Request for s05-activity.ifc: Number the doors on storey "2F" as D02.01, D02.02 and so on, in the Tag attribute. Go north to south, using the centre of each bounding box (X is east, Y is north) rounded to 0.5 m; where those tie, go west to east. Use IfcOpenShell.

First a look at what the model holds.

```python
import ifcopenshell
import ifcopenshell.util.element
import ifcopenshell.util.placement

model = ifcopenshell.open("s05-activity.ifc")
print(model.schema)
storey = next(s for s in model.by_type("IfcBuildingStorey") if s.Name == "2F")
doors = [e for e in ifcopenshell.util.element.get_decomposition(storey) if e.is_a("IfcDoor")]
for e in sorted(doors, key=lambda e: e.id()):
    origin = ifcopenshell.util.placement.get_local_placement(e.ObjectPlacement)[:3, 3]
    print(e.id(), e.Tag, e.Name, origin.round(2) + 0.0, sep=" | ")
```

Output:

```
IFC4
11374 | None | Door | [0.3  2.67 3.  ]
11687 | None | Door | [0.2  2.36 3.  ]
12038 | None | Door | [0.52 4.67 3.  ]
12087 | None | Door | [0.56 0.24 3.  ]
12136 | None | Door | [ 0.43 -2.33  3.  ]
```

```python
import ifcopenshell
import ifcopenshell.geom
import ifcopenshell.util.element
import ifcopenshell.util.shape

model = ifcopenshell.open("s05-activity.ifc")
settings = ifcopenshell.geom.settings()
settings.set("use-world-coords", True)


def centre(element):
    shape = ifcopenshell.geom.create_shape(settings, element)
    return ifcopenshell.util.shape.get_bbox_centroid(shape.geometry)


storey = next(s for s in model.by_type("IfcBuildingStorey") if s.Name == "2F")
doors = [e for e in ifcopenshell.util.element.get_decomposition(storey) if e.is_a("IfcDoor")]

# Insertion points can sit at a corner or the storey origin, so sort by the geometry (in metres).
centres = {e: centre(e) for e in doors}
doors.sort(key=lambda e: (-round(centres[e][1] / 0.5), centres[e][0]))

for i, e in enumerate(doors, start=1):
    number = f"D02.{i:02d}"
    e.Tag = number
    print(e.id(), number)

model.write("s05-activity-out.ifc")
```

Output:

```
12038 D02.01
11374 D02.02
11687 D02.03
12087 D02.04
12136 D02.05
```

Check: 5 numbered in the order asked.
